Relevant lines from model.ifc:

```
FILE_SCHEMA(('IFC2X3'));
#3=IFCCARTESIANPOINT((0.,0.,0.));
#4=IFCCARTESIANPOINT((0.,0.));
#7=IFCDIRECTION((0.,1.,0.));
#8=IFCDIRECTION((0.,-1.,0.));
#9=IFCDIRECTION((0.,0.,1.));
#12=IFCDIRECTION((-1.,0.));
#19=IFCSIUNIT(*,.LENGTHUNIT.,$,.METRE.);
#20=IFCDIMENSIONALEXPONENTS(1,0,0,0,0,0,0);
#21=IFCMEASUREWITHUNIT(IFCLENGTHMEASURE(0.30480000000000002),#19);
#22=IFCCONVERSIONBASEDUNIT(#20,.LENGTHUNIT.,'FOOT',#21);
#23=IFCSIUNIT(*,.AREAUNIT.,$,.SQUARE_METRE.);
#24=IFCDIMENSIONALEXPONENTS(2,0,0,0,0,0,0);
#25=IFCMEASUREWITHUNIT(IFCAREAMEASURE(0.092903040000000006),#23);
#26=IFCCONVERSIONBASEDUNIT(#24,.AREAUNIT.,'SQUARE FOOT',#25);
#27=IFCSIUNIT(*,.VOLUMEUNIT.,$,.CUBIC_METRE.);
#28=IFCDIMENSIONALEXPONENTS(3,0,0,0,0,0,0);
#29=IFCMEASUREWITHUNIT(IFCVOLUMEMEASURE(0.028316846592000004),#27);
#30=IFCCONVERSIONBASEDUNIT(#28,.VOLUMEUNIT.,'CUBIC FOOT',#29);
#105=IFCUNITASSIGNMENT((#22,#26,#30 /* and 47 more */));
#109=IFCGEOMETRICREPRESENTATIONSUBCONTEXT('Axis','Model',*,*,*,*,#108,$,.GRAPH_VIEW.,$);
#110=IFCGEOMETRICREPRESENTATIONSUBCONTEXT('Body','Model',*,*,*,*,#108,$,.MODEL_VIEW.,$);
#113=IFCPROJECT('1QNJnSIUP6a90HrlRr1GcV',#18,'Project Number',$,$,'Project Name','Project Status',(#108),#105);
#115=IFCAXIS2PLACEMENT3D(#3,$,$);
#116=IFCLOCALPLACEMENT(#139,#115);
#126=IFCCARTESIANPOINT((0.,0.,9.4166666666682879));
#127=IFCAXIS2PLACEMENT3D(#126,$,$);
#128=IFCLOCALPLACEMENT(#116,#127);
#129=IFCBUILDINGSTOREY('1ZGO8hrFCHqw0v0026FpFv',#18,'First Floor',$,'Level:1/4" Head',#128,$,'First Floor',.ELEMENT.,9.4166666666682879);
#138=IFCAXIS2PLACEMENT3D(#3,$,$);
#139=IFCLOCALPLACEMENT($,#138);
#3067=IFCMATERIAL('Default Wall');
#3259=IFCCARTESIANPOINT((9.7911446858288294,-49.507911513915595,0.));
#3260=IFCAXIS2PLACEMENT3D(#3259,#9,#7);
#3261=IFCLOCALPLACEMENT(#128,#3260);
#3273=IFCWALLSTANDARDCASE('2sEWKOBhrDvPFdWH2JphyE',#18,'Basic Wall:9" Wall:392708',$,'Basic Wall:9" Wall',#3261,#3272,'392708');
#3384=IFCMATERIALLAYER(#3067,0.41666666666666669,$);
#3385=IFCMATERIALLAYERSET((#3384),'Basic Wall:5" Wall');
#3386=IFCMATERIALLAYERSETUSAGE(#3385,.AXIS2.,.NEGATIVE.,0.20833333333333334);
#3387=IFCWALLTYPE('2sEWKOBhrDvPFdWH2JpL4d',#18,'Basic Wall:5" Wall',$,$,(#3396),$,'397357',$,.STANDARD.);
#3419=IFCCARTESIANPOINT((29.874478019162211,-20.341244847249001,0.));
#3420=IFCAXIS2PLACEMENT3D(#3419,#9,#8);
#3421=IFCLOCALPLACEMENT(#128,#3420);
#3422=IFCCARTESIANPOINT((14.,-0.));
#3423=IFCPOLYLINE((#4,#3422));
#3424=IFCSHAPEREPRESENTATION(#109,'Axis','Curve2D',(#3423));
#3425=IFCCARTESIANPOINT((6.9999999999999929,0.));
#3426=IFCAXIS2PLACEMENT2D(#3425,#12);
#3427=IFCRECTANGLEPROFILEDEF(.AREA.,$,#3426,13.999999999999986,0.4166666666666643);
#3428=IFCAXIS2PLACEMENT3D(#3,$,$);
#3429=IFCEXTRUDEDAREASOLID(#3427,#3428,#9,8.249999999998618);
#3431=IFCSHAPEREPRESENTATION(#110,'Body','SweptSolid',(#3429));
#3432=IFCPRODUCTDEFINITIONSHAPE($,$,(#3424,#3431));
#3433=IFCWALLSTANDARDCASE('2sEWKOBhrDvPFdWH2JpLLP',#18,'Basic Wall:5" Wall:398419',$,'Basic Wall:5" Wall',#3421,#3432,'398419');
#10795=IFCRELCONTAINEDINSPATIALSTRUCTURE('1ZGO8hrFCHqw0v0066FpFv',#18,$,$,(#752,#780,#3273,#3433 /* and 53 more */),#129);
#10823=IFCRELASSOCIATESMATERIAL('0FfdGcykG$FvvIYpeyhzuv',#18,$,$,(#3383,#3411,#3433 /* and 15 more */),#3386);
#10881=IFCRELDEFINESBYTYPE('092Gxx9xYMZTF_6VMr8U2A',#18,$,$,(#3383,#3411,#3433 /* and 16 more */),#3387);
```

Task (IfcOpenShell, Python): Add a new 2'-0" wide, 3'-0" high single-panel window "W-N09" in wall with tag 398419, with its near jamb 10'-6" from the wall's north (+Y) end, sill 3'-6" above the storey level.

```python
import numpy as np
import ifcopenshell
import ifcopenshell.api.feature
import ifcopenshell.api.geometry
import ifcopenshell.api.root
import ifcopenshell.api.spatial
import ifcopenshell.api.type
import ifcopenshell.geom
import ifcopenshell.util.element
import ifcopenshell.util.placement
import ifcopenshell.util.representation
import ifcopenshell.util.shape
import ifcopenshell.util.unit

model = ifcopenshell.open("model.ifc")
unit_scale = ifcopenshell.util.unit.calculate_unit_scale(model)
settings = ifcopenshell.geom.settings()


def volume(element):
    """Net volume in cubic metres, openings subtracted."""
    shape = ifcopenshell.geom.create_shape(settings, element)
    return ifcopenshell.util.shape.get_volume(shape.geometry)


wall = model.by_guid("2sEWKOBhrDvPFdWH2JpLLP")
storey = ifcopenshell.util.element.get_container(wall, ifc_class="IfcBuildingStorey")
context = ifcopenshell.util.representation.get_context(model, "Model", "Body", "MODEL_VIEW")
before = volume(wall)

width, height, from_end, sill = 0.6096, 0.9144, 3.2004, 1.0668  # metres

# The wall runs along its own X axis, and the end named is its -X end.
wall_shape = ifcopenshell.geom.create_shape(settings, wall)
x, y, z = ifcopenshell.util.shape.get_vertices(wall_shape.geometry).T
start = x.min() + from_end
face, thickness = float(y.min()), float(y.max() - y.min())
wall_matrix = ifcopenshell.util.placement.get_local_placement(wall.ObjectPlacement)
level = ifcopenshell.util.placement.get_local_placement(storey.ObjectPlacement)[2, 3]


def in_wall(x, y):
    """Placement at x, y metres in the wall's axes, at sill height."""
    matrix = wall_matrix.copy()
    matrix[:, 3] = wall_matrix @ np.array([x / unit_scale, y / unit_scale, 0.0, 1.0])
    matrix[2, 3] = level + sill / unit_scale
    return matrix


# Opening: a box that overshoots both wall faces by 50 mm.
opening = ifcopenshell.api.root.create_entity(model, ifc_class="IfcOpeningElement")
box = ifcopenshell.api.geometry.add_wall_representation(
    model, context=context, length=width, height=height, thickness=thickness + 0.1
)
ifcopenshell.api.geometry.assign_representation(model, product=opening, representation=box)
ifcopenshell.api.geometry.edit_object_placement(model, product=opening, matrix=in_wall(start, face - 0.05), is_si=False)
ifcopenshell.api.feature.add_feature(model, feature=opening, element=wall)

window = ifcopenshell.api.root.create_entity(model, ifc_class="IfcWindow", name="W-N09")
window.OverallWidth, window.OverallHeight = width / unit_scale, height / unit_scale
body = ifcopenshell.api.geometry.add_window_representation(
    model,
    context=context,
    overall_width=window.OverallWidth,
    overall_height=window.OverallHeight,
    partition_type="SINGLE_PANEL",
)
ifcopenshell.api.geometry.assign_representation(model, product=window, representation=body)
ifcopenshell.api.spatial.assign_container(model, products=[window], relating_structure=storey)
fills = ifcopenshell.api.feature.add_filling(model, opening=opening, element=window)
fills.OwnerHistory = window.OwnerHistory  # required in IFC2X3

# IFC2X3 keeps the operation on the window style.
style = ifcopenshell.api.root.create_entity(model, ifc_class="IfcWindowStyle", name="W-N09")
style.OperationType, style.ConstructionType = "SINGLE_PANEL", "NOTDEFINED"
style.ParameterTakesPrecedence = style.Sizeable = False
ifcopenshell.api.type.assign_type(model, related_objects=[window], relating_type=style)

# Centre the window in the wall's thickness.
ifcopenshell.api.geometry.edit_object_placement(model, product=window, matrix=in_wall(start, face), is_si=False)
window_shape = ifcopenshell.geom.create_shape(settings, window)
depth = ifcopenshell.util.shape.get_vertices(window_shape.geometry)[:, 1]
offset = face + thickness / 2 - (depth.min() + depth.max()) / 2
ifcopenshell.api.geometry.edit_object_placement(model, product=window, matrix=in_wall(start, offset), is_si=False)

after = volume(wall)

print(f"wall volume {before:.3f} -> {after:.3f} m3")

model.write("model-out.ifc")
```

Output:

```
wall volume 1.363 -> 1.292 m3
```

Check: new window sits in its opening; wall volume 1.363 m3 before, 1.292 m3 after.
